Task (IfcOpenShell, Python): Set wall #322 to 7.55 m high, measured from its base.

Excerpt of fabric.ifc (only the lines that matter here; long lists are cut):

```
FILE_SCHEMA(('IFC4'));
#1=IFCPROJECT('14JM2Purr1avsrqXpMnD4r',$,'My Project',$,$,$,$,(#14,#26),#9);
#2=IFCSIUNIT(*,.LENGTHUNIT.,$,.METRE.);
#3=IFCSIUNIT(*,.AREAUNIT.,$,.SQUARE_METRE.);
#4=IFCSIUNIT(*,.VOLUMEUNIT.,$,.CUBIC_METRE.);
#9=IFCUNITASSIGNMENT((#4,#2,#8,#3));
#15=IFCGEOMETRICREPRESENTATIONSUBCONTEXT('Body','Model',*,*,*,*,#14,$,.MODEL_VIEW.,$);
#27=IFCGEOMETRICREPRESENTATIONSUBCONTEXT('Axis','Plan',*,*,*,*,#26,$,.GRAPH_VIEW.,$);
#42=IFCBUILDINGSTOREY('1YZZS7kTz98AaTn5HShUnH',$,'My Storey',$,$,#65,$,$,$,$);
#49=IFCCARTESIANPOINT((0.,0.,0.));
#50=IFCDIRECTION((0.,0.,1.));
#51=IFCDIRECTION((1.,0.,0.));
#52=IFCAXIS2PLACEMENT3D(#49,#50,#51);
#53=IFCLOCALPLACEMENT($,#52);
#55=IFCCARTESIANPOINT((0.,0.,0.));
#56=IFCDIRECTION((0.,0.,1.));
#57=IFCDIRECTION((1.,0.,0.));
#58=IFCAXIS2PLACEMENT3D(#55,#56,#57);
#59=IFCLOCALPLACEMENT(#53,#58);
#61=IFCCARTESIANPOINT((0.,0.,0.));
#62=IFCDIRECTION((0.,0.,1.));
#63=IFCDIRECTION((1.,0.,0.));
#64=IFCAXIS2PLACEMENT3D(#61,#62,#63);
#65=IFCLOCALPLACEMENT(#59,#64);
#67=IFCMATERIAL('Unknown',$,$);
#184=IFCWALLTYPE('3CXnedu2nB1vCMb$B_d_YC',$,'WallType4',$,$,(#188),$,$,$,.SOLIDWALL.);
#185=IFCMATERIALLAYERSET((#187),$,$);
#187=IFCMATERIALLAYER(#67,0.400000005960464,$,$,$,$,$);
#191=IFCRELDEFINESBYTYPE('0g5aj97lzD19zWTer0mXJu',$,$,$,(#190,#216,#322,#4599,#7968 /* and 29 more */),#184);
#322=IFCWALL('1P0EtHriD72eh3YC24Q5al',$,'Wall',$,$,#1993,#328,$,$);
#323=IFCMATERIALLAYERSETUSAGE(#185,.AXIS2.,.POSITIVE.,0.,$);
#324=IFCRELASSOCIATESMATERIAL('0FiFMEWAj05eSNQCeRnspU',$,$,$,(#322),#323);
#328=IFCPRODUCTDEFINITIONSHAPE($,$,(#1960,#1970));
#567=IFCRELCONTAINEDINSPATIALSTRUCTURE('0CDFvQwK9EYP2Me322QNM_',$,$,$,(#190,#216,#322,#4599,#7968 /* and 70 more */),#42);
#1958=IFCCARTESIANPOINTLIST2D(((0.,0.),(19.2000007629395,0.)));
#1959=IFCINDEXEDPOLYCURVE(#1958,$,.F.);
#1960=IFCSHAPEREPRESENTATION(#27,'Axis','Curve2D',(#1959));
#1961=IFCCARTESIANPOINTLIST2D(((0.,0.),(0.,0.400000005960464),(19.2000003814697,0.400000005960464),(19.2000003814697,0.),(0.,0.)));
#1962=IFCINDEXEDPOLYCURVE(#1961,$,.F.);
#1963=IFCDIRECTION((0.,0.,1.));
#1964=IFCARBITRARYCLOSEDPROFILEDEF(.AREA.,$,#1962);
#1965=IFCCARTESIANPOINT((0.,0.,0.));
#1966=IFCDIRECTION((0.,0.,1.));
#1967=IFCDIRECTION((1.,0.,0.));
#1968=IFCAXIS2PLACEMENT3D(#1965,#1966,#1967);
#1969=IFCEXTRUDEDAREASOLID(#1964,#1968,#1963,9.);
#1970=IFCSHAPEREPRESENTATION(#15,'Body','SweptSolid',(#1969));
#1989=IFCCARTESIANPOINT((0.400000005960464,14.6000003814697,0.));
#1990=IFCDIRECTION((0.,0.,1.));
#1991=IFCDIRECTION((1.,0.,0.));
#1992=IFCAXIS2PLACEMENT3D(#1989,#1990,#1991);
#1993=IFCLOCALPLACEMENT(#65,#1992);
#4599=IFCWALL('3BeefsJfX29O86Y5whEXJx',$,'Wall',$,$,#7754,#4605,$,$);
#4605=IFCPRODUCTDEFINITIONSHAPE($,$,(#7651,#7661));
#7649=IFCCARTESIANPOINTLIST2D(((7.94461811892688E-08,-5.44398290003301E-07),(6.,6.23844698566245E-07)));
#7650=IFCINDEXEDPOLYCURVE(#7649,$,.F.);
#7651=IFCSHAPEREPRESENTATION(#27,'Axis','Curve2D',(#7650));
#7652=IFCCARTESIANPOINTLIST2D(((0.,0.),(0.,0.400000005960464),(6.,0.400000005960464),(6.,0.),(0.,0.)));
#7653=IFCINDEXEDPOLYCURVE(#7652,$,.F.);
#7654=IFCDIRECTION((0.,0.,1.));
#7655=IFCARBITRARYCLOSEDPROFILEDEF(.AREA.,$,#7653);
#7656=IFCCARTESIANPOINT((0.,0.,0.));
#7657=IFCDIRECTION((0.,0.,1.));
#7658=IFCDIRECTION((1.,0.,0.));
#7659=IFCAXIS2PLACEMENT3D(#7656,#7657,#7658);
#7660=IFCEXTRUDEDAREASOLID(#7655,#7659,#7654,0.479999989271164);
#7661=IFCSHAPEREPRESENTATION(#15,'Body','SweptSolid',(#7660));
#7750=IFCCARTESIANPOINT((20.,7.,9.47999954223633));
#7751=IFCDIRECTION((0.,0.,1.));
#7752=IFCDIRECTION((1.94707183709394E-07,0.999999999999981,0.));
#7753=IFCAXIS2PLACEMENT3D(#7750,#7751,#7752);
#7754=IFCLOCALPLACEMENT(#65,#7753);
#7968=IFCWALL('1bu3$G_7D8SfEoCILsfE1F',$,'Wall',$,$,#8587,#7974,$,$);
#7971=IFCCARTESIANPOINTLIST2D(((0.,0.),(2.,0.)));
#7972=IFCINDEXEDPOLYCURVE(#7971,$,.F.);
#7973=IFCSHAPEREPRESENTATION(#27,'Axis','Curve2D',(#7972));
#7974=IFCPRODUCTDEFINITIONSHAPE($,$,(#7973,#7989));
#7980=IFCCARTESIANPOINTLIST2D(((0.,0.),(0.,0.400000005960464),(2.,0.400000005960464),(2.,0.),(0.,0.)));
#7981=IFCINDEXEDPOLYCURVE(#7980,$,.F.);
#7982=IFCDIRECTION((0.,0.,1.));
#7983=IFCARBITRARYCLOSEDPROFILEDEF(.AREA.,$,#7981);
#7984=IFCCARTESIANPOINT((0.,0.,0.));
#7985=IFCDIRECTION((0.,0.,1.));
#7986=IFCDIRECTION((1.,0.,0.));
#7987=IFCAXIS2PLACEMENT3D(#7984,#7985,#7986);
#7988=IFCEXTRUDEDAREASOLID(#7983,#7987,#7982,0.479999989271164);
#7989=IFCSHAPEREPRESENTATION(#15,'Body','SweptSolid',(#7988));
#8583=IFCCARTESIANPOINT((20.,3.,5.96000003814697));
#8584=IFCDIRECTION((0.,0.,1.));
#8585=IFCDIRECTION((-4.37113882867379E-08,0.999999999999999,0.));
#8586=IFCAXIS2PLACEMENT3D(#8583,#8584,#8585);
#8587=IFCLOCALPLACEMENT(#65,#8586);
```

```python
import ifcopenshell
import ifcopenshell.geom
import ifcopenshell.util.representation
import ifcopenshell.util.shape

model = ifcopenshell.open("fabric.ifc")
settings = ifcopenshell.geom.settings()


def volume(element):
    """Net volume in cubic metres, openings subtracted."""
    shape = ifcopenshell.geom.create_shape(settings, element)
    return ifcopenshell.util.shape.get_volume(shape.geometry)


wall = model.by_id(322)
before = volume(wall)

body = ifcopenshell.util.representation.get_representation(wall, "Model", "Body")
solid = body.Items[0]
old_height = solid.Depth
solid.Depth = 7.55
after = volume(wall)

print(f"height {old_height:g} -> {solid.Depth:g}, volume {before:.3f} -> {after:.3f} m3")

model.write("fabric_updated.ifc")
```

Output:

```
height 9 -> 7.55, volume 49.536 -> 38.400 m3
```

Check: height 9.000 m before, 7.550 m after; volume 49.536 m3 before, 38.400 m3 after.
